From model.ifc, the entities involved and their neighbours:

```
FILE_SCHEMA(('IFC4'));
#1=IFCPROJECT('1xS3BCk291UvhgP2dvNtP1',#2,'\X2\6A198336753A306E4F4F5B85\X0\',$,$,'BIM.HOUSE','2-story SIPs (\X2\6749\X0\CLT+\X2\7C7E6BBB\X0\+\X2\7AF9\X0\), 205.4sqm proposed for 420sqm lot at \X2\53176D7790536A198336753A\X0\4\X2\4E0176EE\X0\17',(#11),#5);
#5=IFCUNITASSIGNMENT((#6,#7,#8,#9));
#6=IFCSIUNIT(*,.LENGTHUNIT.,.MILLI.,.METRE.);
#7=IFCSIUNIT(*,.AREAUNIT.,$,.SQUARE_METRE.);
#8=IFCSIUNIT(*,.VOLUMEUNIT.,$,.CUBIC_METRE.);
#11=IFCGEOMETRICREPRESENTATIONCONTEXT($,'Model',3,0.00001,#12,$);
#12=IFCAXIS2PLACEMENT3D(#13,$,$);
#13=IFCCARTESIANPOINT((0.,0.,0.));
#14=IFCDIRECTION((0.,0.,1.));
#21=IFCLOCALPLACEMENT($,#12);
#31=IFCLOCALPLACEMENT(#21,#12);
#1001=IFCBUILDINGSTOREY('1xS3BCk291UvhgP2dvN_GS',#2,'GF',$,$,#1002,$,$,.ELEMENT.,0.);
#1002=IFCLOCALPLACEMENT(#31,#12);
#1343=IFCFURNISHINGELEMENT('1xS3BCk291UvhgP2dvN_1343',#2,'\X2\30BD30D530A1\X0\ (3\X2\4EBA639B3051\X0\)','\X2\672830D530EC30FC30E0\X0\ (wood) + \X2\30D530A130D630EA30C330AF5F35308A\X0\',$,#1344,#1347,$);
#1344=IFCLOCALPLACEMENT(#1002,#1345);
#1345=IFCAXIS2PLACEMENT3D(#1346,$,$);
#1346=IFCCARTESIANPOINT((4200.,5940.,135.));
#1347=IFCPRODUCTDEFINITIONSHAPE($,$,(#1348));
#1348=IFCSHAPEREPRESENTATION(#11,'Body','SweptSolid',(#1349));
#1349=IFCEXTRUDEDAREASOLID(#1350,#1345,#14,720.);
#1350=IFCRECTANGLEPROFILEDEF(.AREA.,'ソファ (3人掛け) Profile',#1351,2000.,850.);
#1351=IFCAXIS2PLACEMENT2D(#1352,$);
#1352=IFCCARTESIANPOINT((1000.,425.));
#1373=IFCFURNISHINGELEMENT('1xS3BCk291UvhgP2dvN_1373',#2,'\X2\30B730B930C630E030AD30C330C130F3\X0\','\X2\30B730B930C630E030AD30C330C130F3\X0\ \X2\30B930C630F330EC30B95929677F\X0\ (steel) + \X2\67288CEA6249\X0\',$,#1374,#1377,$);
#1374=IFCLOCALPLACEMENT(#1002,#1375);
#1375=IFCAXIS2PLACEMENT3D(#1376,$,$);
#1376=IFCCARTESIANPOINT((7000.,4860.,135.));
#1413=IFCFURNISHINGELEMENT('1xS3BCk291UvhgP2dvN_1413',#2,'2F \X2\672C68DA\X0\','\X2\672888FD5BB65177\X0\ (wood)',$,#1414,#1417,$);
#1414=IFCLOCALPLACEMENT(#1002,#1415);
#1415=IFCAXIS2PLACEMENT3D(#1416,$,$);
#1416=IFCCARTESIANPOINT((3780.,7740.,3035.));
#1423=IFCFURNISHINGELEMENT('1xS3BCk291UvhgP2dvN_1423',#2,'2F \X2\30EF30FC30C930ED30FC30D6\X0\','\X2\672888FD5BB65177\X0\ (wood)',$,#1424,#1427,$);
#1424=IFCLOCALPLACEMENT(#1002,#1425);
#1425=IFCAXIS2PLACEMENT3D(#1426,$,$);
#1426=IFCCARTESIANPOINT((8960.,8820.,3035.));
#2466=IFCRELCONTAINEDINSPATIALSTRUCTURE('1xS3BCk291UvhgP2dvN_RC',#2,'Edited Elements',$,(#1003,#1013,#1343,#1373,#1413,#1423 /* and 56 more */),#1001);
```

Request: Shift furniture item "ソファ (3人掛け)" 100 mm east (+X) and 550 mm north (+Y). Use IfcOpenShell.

```python
import ifcopenshell
import ifcopenshell.api.geometry
import ifcopenshell.util.placement
import ifcopenshell.util.unit

model = ifcopenshell.open("model.ifc")
unit_scale = ifcopenshell.util.unit.calculate_unit_scale(model)

item = model.by_guid("1xS3BCk291UvhgP2dvN_1343")
matrix = ifcopenshell.util.placement.get_local_placement(item.ObjectPlacement)
matrix[0, 3] += 0.1 / unit_scale
matrix[1, 3] += 0.55 / unit_scale
ifcopenshell.api.geometry.edit_object_placement(model, product=item, matrix=matrix, is_si=False)

print(ifcopenshell.util.placement.get_local_placement(item.ObjectPlacement).round(3) + 0.0)

model.write("model_updated.ifc")
```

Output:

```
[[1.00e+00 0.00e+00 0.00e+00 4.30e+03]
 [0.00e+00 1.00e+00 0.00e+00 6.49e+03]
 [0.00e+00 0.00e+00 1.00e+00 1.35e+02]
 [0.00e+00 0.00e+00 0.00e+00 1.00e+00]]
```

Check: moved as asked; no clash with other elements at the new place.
